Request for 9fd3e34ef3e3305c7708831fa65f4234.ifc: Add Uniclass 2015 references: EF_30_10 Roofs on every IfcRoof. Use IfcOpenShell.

First a look at what the model holds.

```python
import ifcopenshell

model = ifcopenshell.open("9fd3e34ef3e3305c7708831fa65f4234.ifc")
print(model.schema)
print("classifications:", [c.Name for c in model.by_type("IfcClassification")])
for ifc_class in ("IfcDoor", "IfcRoof", "IfcStair", "IfcWall", "IfcWindow"):
    print(ifc_class, len(model.by_type(ifc_class)))
```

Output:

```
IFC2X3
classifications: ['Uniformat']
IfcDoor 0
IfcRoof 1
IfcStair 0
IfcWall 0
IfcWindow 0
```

```python
import ifcopenshell
import ifcopenshell.api.classification

model = ifcopenshell.open("9fd3e34ef3e3305c7708831fa65f4234.ifc")

# IFC2X3 requires Source and Edition and has no link from the project to the system.
system = model.create_entity("IfcClassification", Source="NBS", Edition="2015", Name="Uniclass 2015")

codes = {
    "IfcRoof": ("EF_30_10", "Roofs"),
}
for ifc_class, (code, name) in codes.items():
    products = model.by_type(ifc_class)
    ifcopenshell.api.classification.add_reference(
        model, products=products, classification=system, identification=code, name=name
    )
    print(code, len(products))

model.write("9fd3e34ef3e3305c7708831fa65f4234_rev.ifc")
```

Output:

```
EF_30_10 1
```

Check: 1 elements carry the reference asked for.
